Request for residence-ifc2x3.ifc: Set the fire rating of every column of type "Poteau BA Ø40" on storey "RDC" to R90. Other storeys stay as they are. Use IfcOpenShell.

First a look at what the model holds.

```python
import ifcopenshell
import ifcopenshell.util.element

model = ifcopenshell.open("residence-ifc2x3.ifc")
print(model.schema)
storey = next(s for s in model.by_type("IfcBuildingStorey") if s.Name == "RDC")
columns = [e for e in ifcopenshell.util.element.get_decomposition(storey) if e.is_a("IfcColumn")]
seen = {}
for e in columns:
    element_type = ifcopenshell.util.element.get_type(e)
    key = (element_type.Name if element_type != e and element_type else None, ifcopenshell.util.element.get_pset(e, "Pset_ColumnCommon", "FireRating"))
    seen[key] = seen.get(key, 0) + 1
for (name, value), count in sorted(seen.items(), key=str):
    print(count, "x", name, "|", value)
```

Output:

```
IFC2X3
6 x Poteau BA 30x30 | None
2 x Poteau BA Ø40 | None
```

```python
import ifcopenshell
import ifcopenshell.api.pset
import ifcopenshell.util.element

model = ifcopenshell.open("residence-ifc2x3.ifc")

storey = next(s for s in model.by_type("IfcBuildingStorey") if s.Name == "RDC")
columns = [e for e in ifcopenshell.util.element.get_decomposition(storey) if e.is_a("IfcColumn")]

count = 0
for e in columns:
    element_type = ifcopenshell.util.element.get_type(e)
    if element_type in (None, e) or element_type.Name != "Poteau BA Ø40":
        continue
    # add_pset returns the element's existing set when there is one.
    pset = ifcopenshell.api.pset.add_pset(model, product=e, name="Pset_ColumnCommon")
    ifcopenshell.api.pset.edit_pset(model, pset=pset, properties={"FireRating": "R90"})
    count += 1

print(count, "columns updated")

model.write("residence-ifc2x3-out.ifc")
```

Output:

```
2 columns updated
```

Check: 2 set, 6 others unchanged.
